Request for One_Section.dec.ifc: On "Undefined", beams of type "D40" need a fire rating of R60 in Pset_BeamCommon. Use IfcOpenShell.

First a look at what the model holds.

```python
import ifcopenshell
import ifcopenshell.util.element

model = ifcopenshell.open("One_Section.dec.ifc")
print(model.schema)
storey = next(s for s in model.by_type("IfcBuildingStorey") if s.Name == "Undefined")
beams = [e for e in ifcopenshell.util.element.get_decomposition(storey) if e.is_a("IfcBeam")]
seen = {}
for e in beams:
    element_type = ifcopenshell.util.element.get_type(e)
    key = (element_type.Name if element_type != e and element_type else None, ifcopenshell.util.element.get_pset(e, "Pset_BeamCommon", "FireRating"))
    seen[key] = seen.get(key, 0) + 1
for (name, value), count in sorted(seen.items(), key=str):
    print(count, "x", name, "|", value)
```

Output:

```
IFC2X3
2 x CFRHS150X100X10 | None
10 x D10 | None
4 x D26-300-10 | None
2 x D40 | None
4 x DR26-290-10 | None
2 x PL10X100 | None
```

```python
import ifcopenshell
import ifcopenshell.api.pset
import ifcopenshell.util.element

model = ifcopenshell.open("One_Section.dec.ifc")

storey = next(s for s in model.by_type("IfcBuildingStorey") if s.Name == "Undefined")
beams = [e for e in ifcopenshell.util.element.get_decomposition(storey) if e.is_a("IfcBeam")]

count = 0
for e in beams:
    element_type = ifcopenshell.util.element.get_type(e)
    if element_type in (None, e) or element_type.Name != "D40":
        continue
    found = ifcopenshell.util.element.get_pset(e, "Pset_BeamCommon", should_inherit=False)
    if found:
        pset = model.by_id(found["id"])
        if len(ifcopenshell.util.element.get_elements_by_pset(pset)) > 1:
            pset = ifcopenshell.api.pset.unshare_pset(model, products=[e], pset=pset)[0]
    else:
        pset = ifcopenshell.api.pset.add_pset(model, product=e, name="Pset_BeamCommon")
    ifcopenshell.api.pset.edit_pset(model, pset=pset, properties={"FireRating": "R60"})
    count += 1

print(count, "beams updated")

model.write("One_Section.dec_rev.ifc")
```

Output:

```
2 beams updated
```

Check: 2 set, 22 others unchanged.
